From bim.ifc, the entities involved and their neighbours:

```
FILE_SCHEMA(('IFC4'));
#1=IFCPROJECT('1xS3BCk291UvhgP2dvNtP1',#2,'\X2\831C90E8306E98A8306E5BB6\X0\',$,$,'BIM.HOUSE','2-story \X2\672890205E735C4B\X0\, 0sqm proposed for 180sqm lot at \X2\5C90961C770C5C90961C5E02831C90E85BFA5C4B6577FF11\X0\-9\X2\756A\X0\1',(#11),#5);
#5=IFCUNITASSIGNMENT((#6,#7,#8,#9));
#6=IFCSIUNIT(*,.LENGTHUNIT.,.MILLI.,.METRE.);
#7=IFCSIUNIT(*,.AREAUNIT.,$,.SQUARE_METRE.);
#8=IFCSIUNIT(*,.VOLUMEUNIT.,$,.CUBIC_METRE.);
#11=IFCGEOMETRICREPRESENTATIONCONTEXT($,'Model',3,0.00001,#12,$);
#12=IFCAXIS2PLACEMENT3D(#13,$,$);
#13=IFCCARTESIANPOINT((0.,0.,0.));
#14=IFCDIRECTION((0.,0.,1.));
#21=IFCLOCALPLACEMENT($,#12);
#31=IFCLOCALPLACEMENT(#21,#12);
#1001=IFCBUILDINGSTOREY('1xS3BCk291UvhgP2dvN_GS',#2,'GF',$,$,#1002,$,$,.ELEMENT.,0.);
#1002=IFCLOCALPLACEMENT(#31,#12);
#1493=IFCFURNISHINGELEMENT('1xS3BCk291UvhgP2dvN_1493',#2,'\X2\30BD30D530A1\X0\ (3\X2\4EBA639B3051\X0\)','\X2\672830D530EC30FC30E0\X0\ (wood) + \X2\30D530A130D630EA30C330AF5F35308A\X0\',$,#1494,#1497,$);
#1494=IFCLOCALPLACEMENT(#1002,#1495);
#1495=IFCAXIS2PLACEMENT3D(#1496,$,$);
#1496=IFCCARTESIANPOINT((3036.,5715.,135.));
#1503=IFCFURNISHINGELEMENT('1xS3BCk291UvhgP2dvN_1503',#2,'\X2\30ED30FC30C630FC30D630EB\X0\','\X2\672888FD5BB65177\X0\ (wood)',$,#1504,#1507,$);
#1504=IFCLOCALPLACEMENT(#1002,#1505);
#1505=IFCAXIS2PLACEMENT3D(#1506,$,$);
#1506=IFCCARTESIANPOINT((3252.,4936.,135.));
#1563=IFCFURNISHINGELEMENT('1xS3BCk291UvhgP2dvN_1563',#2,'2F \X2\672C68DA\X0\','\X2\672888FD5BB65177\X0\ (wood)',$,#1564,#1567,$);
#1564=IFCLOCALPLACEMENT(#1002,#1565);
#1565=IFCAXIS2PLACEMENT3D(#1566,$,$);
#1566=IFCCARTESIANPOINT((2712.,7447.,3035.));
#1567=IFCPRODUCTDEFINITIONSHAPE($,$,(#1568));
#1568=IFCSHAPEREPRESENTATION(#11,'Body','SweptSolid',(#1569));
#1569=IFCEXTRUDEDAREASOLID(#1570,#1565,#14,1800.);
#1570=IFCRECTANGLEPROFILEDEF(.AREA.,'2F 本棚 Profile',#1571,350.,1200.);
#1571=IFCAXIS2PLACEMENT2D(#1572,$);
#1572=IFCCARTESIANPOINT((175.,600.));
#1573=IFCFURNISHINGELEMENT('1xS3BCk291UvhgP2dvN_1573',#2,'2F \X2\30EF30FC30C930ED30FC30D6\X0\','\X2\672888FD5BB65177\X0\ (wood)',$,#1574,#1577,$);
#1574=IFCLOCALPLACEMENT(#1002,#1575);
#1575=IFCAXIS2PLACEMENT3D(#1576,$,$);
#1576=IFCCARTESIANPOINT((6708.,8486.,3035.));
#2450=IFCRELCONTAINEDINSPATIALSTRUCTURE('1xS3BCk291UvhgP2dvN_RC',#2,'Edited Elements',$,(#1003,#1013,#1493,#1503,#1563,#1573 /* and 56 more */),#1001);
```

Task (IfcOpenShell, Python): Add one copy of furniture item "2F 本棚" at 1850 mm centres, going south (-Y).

```python
import numpy as np
import ifcopenshell
import ifcopenshell.api.geometry
import ifcopenshell.api.root
import ifcopenshell.util.element
import ifcopenshell.util.placement

model = ifcopenshell.open("bim.ifc")


def reuse_history(source, copy):
    """copy_class also copies each property set's owner history, people and application; keep the originals."""
    for rel in copy.IsDefinedBy:
        if rel.is_a("IfcRelDefinesByProperties") and (history := rel.RelatingPropertyDefinition.OwnerHistory):
            rel.RelatingPropertyDefinition.OwnerHistory = source.OwnerHistory
            ifcopenshell.util.element.remove_deep2(model, history)


source = model.by_guid("1xS3BCk291UvhgP2dvN_1563")
base = ifcopenshell.util.placement.get_local_placement(source.ObjectPlacement)
step = np.array([0.0, -1.0, 0.0]) * 1850.0

for i in range(1, 2):
    copy = ifcopenshell.api.root.copy_class(model, product=source)
    copy.Representation = ifcopenshell.util.element.copy_deep(
        model, source.Representation, exclude=["IfcGeometricRepresentationContext", "IfcRepresentationMap"]
    )
    reuse_history(source, copy)
    matrix = base.copy()
    matrix[:3, 3] += i * step
    print("added at", matrix[:3, 3].round(3) + 0.0)
    ifcopenshell.api.geometry.edit_object_placement(model, product=copy, matrix=matrix, is_si=False)

model.write("bim_rev.ifc")
```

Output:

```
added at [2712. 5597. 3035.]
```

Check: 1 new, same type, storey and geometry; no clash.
